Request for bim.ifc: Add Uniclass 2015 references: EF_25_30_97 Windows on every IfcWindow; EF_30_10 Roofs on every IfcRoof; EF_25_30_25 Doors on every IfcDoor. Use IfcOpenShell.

First a look at what the model holds.

```python
import ifcopenshell

model = ifcopenshell.open("bim.ifc")
print(model.schema)
print("classifications:", [c.Name for c in model.by_type("IfcClassification")])
for ifc_class in ("IfcDoor", "IfcRoof", "IfcStair", "IfcWall", "IfcWindow"):
    print(ifc_class, len(model.by_type(ifc_class)))
```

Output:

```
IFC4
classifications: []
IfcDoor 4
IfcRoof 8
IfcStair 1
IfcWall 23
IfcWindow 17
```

```python
import ifcopenshell
import ifcopenshell.api.classification

model = ifcopenshell.open("bim.ifc")

system = ifcopenshell.api.classification.add_classification(model, classification="Uniclass 2015")

codes = {
    "IfcWindow": ("EF_25_30_97", "Windows"),
    "IfcRoof": ("EF_30_10", "Roofs"),
    "IfcDoor": ("EF_25_30_25", "Doors"),
}
for ifc_class, (code, name) in codes.items():
    products = model.by_type(ifc_class)
    ifcopenshell.api.classification.add_reference(
        model, products=products, classification=system, identification=code, name=name
    )
    print(code, len(products))

model.write("bim_updated.ifc")
```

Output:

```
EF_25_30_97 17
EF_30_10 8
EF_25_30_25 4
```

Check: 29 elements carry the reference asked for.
